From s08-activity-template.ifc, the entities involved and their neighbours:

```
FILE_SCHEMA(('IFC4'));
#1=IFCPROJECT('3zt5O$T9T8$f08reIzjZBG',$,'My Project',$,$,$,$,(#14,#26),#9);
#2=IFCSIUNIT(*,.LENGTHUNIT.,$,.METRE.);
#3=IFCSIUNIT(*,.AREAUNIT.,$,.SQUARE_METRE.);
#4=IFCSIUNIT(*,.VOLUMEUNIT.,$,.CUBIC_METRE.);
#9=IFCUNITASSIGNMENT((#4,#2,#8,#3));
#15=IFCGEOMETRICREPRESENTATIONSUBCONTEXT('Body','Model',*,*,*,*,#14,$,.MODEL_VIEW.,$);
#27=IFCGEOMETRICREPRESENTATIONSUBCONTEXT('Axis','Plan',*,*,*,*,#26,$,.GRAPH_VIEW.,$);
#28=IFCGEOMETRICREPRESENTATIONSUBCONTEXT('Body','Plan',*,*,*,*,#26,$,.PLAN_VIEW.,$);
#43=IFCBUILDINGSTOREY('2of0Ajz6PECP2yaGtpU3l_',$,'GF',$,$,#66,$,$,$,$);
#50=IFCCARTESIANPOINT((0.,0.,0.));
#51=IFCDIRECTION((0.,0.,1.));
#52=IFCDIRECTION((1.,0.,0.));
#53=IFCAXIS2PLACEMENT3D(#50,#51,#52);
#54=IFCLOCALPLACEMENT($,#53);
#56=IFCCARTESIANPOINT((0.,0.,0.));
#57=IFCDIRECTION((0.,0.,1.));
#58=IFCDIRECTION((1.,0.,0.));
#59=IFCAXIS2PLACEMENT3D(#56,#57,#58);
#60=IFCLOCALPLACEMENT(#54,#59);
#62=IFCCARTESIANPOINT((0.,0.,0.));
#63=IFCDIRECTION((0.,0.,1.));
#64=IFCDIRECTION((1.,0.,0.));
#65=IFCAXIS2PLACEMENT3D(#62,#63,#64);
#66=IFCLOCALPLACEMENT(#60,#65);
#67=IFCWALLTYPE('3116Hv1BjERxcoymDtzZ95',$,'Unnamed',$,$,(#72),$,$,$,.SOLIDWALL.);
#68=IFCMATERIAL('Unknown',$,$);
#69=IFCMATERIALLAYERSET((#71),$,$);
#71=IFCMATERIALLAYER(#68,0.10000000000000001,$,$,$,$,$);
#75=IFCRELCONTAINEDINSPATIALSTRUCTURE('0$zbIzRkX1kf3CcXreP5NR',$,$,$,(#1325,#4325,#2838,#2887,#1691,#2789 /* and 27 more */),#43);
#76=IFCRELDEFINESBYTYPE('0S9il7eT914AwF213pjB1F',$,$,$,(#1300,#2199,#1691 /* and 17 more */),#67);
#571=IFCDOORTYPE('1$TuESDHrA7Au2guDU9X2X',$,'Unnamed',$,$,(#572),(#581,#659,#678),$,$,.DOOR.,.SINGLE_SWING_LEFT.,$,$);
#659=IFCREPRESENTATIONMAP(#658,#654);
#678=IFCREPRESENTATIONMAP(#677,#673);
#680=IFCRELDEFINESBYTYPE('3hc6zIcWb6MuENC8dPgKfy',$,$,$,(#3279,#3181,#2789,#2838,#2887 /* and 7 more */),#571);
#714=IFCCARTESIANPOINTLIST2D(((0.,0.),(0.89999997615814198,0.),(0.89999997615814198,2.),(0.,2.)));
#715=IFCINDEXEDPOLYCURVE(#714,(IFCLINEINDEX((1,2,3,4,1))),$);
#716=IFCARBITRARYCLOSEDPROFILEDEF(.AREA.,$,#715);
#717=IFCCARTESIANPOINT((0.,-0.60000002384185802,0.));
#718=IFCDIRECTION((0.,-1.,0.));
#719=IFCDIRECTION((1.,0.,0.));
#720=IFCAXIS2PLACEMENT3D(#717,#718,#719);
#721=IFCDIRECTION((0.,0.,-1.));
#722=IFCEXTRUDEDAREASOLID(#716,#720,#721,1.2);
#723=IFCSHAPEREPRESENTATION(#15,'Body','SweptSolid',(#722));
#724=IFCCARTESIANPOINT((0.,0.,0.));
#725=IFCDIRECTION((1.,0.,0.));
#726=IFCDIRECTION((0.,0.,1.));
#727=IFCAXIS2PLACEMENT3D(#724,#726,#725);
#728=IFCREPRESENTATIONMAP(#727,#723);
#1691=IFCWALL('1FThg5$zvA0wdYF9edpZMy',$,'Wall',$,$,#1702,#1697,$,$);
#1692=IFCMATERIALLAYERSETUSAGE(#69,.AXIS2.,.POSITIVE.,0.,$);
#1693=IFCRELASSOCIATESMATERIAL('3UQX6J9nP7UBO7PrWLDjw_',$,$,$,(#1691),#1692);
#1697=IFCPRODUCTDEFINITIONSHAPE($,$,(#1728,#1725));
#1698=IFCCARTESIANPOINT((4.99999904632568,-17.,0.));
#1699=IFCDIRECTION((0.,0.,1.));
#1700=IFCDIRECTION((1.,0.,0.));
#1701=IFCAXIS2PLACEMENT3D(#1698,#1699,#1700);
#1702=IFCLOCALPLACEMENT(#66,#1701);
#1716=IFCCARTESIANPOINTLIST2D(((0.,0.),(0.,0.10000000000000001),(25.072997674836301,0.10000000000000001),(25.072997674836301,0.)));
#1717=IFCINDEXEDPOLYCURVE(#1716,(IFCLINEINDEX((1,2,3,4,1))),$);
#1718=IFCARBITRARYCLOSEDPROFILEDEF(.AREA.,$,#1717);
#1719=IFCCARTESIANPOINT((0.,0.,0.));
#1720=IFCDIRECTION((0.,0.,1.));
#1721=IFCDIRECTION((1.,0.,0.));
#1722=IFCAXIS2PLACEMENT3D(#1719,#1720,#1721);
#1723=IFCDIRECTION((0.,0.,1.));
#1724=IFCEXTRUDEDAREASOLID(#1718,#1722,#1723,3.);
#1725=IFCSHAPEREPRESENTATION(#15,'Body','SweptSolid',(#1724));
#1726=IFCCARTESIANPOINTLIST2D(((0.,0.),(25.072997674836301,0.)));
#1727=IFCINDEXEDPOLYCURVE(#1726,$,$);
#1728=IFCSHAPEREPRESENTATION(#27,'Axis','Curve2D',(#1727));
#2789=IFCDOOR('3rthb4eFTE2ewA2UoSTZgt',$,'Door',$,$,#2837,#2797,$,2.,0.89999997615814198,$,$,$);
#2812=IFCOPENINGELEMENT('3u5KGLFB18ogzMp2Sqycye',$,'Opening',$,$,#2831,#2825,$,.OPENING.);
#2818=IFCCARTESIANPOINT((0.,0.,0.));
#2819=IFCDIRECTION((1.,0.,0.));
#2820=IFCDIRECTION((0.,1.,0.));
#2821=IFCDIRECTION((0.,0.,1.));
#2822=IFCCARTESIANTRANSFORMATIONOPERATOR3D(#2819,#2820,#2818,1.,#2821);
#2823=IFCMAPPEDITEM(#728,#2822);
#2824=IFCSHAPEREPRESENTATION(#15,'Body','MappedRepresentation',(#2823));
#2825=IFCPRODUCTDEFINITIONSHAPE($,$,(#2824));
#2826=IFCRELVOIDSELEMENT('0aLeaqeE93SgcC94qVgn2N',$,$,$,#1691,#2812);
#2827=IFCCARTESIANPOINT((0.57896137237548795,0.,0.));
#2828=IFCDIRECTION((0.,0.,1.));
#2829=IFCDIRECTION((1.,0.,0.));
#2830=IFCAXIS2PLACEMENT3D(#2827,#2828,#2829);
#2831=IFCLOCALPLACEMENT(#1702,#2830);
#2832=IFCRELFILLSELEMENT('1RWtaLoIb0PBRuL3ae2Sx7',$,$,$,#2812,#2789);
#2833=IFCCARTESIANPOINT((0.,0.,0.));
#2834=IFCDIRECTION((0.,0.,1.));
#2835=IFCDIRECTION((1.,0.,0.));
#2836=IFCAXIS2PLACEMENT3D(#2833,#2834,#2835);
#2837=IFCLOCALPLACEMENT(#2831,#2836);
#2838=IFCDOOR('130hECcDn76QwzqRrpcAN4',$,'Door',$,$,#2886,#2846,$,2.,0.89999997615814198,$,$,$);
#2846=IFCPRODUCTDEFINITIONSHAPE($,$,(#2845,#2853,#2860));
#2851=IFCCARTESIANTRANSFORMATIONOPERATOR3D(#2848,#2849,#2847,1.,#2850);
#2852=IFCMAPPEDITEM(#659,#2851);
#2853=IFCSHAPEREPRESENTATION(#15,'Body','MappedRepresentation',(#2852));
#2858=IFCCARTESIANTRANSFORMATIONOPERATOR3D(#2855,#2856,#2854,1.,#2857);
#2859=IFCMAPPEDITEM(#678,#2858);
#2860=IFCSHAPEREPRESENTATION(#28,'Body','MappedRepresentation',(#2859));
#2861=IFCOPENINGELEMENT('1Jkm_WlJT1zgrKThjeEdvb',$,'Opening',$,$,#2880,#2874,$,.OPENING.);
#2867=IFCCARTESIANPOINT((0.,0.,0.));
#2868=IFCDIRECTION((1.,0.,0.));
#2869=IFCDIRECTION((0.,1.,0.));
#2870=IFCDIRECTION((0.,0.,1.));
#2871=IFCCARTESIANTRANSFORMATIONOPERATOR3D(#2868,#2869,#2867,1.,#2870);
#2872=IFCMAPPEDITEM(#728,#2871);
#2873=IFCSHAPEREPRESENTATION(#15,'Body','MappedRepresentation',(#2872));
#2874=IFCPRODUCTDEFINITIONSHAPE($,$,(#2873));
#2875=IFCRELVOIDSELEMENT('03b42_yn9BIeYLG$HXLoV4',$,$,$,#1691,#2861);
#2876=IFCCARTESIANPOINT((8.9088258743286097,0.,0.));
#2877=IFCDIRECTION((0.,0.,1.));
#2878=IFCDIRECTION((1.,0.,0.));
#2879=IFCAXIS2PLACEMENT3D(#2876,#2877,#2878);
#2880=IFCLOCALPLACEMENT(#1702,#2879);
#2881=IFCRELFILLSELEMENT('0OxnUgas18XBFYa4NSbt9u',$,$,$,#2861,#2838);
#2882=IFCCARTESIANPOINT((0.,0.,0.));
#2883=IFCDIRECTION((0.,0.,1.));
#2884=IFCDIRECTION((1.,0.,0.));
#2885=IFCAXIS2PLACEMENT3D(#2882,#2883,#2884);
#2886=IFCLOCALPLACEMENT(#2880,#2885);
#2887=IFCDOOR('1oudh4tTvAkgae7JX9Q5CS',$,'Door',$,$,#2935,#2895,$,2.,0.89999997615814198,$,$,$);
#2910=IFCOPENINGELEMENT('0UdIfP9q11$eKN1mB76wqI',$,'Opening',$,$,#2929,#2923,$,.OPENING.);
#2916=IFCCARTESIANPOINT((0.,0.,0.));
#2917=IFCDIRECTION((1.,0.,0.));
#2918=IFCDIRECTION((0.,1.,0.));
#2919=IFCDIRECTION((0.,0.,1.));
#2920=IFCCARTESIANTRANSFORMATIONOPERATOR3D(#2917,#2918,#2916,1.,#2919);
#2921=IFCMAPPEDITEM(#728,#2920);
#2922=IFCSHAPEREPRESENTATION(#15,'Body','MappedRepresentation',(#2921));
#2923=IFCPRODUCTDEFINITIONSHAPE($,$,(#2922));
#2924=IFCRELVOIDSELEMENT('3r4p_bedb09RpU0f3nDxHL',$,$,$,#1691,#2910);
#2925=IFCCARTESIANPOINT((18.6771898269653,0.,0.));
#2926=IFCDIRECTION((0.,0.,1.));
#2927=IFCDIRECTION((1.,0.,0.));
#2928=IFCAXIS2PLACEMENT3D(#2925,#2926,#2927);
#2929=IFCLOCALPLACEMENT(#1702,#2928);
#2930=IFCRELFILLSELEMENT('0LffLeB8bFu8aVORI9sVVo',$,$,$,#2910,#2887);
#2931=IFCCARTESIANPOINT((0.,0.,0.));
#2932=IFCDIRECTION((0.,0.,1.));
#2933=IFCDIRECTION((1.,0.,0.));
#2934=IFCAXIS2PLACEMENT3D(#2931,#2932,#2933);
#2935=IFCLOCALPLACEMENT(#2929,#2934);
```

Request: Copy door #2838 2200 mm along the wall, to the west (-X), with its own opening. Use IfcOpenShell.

```python
import ifcopenshell
import ifcopenshell.api.feature
import ifcopenshell.api.geometry
import ifcopenshell.api.root
import ifcopenshell.geom
import ifcopenshell.util.element
import ifcopenshell.util.placement
import ifcopenshell.util.shape
import ifcopenshell.util.unit

model = ifcopenshell.open("s08-activity-template.ifc")
unit_scale = ifcopenshell.util.unit.calculate_unit_scale(model)
settings = ifcopenshell.geom.settings()


def volume(element):
    """Net volume in cubic metres, openings subtracted."""
    shape = ifcopenshell.geom.create_shape(settings, element)
    return ifcopenshell.util.shape.get_volume(shape.geometry)


door = model.by_id(2838)
opening = door.FillsVoids[0].RelatingOpeningElement
wall = opening.VoidsElements[0].RelatingBuildingElement
before = volume(wall)
shift = ifcopenshell.util.placement.get_local_placement(wall.ObjectPlacement)[:3, 0] * -2.2 / unit_scale

# copy_class copies the void relationship, type, container and properties, but no geometry.
new_opening = ifcopenshell.api.root.copy_class(model, product=opening)
new_opening.Representation = ifcopenshell.util.element.copy_deep(
    model, opening.Representation, exclude=["IfcGeometricRepresentationContext", "IfcRepresentationMap"]
)
new_door = ifcopenshell.api.root.copy_class(model, product=door)
new_door.Representation = ifcopenshell.util.element.copy_deep(
    model, door.Representation, exclude=["IfcGeometricRepresentationContext", "IfcRepresentationMap"]
)
ifcopenshell.api.feature.add_filling(model, opening=new_opening, element=new_door)

for old, new in ((opening, new_opening), (door, new_door)):
    matrix = ifcopenshell.util.placement.get_local_placement(old.ObjectPlacement)
    matrix[:3, 3] += shift
    ifcopenshell.api.geometry.edit_object_placement(model, product=new, matrix=matrix, is_si=False)

after = volume(wall)

print(f"wall volume {before:.3f} -> {after:.3f} m3")

model.write("s08-activity-template_updated.ifc")
```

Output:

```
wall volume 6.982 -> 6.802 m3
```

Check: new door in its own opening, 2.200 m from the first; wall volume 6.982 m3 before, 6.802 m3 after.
